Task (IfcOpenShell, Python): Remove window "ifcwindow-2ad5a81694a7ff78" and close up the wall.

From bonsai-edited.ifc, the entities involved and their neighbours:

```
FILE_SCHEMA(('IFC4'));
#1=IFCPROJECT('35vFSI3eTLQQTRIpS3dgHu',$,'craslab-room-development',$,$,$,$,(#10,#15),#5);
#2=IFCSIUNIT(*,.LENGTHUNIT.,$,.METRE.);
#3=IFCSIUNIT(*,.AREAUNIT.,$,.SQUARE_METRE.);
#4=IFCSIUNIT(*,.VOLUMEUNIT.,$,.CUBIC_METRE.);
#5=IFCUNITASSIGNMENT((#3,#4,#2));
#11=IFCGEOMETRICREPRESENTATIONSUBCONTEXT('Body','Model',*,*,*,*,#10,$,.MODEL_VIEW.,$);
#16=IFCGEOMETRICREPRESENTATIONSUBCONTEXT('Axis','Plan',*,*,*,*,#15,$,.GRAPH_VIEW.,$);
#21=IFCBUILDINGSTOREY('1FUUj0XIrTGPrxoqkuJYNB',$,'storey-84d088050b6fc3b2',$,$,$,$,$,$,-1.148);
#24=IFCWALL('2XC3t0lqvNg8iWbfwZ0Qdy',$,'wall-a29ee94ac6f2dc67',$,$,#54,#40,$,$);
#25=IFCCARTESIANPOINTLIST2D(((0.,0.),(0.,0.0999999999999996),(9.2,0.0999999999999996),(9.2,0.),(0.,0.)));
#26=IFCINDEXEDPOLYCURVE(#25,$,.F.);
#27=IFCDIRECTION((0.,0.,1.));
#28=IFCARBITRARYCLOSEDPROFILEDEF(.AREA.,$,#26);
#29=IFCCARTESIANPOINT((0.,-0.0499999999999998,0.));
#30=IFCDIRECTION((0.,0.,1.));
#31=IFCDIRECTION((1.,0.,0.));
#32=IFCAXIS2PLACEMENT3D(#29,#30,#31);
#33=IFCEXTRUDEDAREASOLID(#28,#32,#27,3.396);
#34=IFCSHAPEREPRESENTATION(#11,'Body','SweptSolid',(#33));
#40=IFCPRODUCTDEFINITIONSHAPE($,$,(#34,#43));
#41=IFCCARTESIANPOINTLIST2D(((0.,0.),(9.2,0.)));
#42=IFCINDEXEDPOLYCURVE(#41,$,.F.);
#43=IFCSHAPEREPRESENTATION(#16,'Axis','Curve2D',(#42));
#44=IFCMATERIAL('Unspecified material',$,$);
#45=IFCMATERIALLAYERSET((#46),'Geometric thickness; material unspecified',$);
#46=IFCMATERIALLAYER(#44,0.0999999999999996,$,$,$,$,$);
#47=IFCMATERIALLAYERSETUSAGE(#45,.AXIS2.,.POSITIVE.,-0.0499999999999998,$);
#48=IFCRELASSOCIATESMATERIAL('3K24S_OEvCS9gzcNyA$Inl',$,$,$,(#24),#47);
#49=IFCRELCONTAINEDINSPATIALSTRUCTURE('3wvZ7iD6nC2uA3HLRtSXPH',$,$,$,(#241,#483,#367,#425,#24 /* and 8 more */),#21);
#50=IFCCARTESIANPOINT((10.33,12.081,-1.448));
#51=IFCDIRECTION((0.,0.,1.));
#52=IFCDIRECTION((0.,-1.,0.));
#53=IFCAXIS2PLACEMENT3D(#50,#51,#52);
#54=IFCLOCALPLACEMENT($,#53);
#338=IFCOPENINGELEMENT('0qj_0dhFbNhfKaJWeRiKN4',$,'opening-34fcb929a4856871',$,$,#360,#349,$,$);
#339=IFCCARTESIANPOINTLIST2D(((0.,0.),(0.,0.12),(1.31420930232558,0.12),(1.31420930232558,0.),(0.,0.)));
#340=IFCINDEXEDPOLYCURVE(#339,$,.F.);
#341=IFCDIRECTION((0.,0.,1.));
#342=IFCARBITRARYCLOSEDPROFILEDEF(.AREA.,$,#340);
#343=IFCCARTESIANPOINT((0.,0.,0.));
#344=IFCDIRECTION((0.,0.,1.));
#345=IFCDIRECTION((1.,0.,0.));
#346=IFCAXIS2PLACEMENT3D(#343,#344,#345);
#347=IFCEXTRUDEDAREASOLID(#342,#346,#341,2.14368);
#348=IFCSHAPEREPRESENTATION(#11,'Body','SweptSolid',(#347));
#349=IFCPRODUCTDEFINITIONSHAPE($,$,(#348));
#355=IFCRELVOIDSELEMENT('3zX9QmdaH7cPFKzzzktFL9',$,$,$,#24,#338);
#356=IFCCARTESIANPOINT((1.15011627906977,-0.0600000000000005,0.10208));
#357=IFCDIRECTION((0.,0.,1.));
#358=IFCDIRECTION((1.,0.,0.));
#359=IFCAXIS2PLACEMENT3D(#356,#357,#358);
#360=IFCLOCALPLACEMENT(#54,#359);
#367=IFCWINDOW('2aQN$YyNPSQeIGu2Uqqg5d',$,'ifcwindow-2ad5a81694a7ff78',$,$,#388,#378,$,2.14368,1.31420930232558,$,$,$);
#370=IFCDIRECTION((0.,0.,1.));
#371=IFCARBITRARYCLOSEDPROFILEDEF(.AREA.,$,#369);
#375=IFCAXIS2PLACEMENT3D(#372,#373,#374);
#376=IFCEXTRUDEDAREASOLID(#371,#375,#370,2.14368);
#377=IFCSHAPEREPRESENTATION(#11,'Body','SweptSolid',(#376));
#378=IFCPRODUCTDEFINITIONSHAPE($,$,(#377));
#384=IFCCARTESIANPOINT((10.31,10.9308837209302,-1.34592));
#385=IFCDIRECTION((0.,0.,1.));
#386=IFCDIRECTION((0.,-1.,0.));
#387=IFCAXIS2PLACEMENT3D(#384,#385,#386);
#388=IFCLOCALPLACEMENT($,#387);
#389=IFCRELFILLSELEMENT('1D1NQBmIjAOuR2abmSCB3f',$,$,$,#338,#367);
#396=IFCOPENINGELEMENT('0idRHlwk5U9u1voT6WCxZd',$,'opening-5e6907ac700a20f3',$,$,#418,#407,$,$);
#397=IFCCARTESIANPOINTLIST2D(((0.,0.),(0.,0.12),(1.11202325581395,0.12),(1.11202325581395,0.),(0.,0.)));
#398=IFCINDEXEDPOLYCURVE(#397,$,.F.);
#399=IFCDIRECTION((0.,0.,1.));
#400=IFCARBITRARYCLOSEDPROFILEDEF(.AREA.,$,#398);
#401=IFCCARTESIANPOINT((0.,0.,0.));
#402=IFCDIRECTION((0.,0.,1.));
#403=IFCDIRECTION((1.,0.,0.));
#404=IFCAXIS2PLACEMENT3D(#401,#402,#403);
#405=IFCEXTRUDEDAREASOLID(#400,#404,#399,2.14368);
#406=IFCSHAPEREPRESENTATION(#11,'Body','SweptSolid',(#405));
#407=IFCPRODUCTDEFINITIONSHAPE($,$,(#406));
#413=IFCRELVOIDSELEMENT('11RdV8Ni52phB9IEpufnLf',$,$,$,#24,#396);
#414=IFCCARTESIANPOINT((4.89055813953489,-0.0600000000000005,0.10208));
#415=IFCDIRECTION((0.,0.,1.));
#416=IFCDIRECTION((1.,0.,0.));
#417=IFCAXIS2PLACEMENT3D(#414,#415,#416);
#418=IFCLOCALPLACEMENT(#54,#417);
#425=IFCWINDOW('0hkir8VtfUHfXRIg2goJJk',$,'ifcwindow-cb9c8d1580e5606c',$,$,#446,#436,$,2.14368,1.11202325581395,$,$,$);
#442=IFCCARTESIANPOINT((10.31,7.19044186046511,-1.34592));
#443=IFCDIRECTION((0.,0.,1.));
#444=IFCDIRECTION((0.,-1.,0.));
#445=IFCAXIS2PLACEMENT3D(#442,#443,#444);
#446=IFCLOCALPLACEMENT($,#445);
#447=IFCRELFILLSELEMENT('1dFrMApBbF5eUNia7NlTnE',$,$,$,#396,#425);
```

```python
import ifcopenshell
import ifcopenshell.api.feature
import ifcopenshell.api.root
import ifcopenshell.geom
import ifcopenshell.util.shape

model = ifcopenshell.open("bonsai-edited.ifc")
settings = ifcopenshell.geom.settings()


def volume(element):
    """Net volume in cubic metres, openings subtracted."""
    shape = ifcopenshell.geom.create_shape(settings, element)
    return ifcopenshell.util.shape.get_volume(shape.geometry)


window = model.by_guid("2aQN$YyNPSQeIGu2Uqqg5d")
opening = window.FillsVoids[0].RelatingOpeningElement
wall = opening.VoidsElements[0].RelatingBuildingElement
before = volume(wall)

ifcopenshell.api.root.remove_product(model, product=window)
ifcopenshell.api.feature.remove_feature(model, feature=opening)

after = volume(wall)

print(f"wall volume {before:.3f} -> {after:.3f} m3")

model.write("bonsai-edited-out.ifc")
```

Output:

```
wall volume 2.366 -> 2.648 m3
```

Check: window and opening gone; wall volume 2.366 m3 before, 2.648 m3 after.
